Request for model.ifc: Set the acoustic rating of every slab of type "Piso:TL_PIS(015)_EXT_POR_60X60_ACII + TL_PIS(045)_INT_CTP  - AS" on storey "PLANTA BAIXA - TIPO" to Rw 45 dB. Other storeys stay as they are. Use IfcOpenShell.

First a look at what the model holds.

```python
import ifcopenshell
import ifcopenshell.util.element

model = ifcopenshell.open("model.ifc")
print(model.schema)
storey = next(s for s in model.by_type("IfcBuildingStorey") if s.Name == "PLANTA BAIXA - TIPO")
slabs = [e for e in ifcopenshell.util.element.get_decomposition(storey) if e.is_a("IfcSlab")]
seen = {}
for e in slabs:
    element_type = ifcopenshell.util.element.get_type(e)
    key = (element_type.Name if element_type != e and element_type else None, ifcopenshell.util.element.get_pset(e, "Pset_SlabCommon", "AcousticRating"))
    seen[key] = seen.get(key, 0) + 1
for (name, value), count in sorted(seen.items(), key=str):
    print(count, "x", name, "|", value)
```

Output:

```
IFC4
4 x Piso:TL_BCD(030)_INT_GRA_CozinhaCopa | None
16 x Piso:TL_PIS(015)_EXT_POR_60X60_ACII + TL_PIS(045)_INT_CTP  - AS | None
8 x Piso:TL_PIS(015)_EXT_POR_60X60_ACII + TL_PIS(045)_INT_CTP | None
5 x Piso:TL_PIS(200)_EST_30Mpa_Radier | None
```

```python
import ifcopenshell
import ifcopenshell.api.pset
import ifcopenshell.util.element

model = ifcopenshell.open("model.ifc")

storey = next(s for s in model.by_type("IfcBuildingStorey") if s.Name == "PLANTA BAIXA - TIPO")
slabs = [e for e in ifcopenshell.util.element.get_decomposition(storey) if e.is_a("IfcSlab")]

count = 0
for e in slabs:
    element_type = ifcopenshell.util.element.get_type(e)
    if element_type in (None, e) or element_type.Name != "Piso:TL_PIS(015)_EXT_POR_60X60_ACII + TL_PIS(045)_INT_CTP  - AS":
        continue
    # add_pset returns the element's existing set when there is one.
    pset = ifcopenshell.api.pset.add_pset(model, product=e, name="Pset_SlabCommon")
    ifcopenshell.api.pset.edit_pset(model, pset=pset, properties={"AcousticRating": "Rw 45 dB"})
    count += 1

print(count, "slabs updated")

model.write("model_v2.ifc")
```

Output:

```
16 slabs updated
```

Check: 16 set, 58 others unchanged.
